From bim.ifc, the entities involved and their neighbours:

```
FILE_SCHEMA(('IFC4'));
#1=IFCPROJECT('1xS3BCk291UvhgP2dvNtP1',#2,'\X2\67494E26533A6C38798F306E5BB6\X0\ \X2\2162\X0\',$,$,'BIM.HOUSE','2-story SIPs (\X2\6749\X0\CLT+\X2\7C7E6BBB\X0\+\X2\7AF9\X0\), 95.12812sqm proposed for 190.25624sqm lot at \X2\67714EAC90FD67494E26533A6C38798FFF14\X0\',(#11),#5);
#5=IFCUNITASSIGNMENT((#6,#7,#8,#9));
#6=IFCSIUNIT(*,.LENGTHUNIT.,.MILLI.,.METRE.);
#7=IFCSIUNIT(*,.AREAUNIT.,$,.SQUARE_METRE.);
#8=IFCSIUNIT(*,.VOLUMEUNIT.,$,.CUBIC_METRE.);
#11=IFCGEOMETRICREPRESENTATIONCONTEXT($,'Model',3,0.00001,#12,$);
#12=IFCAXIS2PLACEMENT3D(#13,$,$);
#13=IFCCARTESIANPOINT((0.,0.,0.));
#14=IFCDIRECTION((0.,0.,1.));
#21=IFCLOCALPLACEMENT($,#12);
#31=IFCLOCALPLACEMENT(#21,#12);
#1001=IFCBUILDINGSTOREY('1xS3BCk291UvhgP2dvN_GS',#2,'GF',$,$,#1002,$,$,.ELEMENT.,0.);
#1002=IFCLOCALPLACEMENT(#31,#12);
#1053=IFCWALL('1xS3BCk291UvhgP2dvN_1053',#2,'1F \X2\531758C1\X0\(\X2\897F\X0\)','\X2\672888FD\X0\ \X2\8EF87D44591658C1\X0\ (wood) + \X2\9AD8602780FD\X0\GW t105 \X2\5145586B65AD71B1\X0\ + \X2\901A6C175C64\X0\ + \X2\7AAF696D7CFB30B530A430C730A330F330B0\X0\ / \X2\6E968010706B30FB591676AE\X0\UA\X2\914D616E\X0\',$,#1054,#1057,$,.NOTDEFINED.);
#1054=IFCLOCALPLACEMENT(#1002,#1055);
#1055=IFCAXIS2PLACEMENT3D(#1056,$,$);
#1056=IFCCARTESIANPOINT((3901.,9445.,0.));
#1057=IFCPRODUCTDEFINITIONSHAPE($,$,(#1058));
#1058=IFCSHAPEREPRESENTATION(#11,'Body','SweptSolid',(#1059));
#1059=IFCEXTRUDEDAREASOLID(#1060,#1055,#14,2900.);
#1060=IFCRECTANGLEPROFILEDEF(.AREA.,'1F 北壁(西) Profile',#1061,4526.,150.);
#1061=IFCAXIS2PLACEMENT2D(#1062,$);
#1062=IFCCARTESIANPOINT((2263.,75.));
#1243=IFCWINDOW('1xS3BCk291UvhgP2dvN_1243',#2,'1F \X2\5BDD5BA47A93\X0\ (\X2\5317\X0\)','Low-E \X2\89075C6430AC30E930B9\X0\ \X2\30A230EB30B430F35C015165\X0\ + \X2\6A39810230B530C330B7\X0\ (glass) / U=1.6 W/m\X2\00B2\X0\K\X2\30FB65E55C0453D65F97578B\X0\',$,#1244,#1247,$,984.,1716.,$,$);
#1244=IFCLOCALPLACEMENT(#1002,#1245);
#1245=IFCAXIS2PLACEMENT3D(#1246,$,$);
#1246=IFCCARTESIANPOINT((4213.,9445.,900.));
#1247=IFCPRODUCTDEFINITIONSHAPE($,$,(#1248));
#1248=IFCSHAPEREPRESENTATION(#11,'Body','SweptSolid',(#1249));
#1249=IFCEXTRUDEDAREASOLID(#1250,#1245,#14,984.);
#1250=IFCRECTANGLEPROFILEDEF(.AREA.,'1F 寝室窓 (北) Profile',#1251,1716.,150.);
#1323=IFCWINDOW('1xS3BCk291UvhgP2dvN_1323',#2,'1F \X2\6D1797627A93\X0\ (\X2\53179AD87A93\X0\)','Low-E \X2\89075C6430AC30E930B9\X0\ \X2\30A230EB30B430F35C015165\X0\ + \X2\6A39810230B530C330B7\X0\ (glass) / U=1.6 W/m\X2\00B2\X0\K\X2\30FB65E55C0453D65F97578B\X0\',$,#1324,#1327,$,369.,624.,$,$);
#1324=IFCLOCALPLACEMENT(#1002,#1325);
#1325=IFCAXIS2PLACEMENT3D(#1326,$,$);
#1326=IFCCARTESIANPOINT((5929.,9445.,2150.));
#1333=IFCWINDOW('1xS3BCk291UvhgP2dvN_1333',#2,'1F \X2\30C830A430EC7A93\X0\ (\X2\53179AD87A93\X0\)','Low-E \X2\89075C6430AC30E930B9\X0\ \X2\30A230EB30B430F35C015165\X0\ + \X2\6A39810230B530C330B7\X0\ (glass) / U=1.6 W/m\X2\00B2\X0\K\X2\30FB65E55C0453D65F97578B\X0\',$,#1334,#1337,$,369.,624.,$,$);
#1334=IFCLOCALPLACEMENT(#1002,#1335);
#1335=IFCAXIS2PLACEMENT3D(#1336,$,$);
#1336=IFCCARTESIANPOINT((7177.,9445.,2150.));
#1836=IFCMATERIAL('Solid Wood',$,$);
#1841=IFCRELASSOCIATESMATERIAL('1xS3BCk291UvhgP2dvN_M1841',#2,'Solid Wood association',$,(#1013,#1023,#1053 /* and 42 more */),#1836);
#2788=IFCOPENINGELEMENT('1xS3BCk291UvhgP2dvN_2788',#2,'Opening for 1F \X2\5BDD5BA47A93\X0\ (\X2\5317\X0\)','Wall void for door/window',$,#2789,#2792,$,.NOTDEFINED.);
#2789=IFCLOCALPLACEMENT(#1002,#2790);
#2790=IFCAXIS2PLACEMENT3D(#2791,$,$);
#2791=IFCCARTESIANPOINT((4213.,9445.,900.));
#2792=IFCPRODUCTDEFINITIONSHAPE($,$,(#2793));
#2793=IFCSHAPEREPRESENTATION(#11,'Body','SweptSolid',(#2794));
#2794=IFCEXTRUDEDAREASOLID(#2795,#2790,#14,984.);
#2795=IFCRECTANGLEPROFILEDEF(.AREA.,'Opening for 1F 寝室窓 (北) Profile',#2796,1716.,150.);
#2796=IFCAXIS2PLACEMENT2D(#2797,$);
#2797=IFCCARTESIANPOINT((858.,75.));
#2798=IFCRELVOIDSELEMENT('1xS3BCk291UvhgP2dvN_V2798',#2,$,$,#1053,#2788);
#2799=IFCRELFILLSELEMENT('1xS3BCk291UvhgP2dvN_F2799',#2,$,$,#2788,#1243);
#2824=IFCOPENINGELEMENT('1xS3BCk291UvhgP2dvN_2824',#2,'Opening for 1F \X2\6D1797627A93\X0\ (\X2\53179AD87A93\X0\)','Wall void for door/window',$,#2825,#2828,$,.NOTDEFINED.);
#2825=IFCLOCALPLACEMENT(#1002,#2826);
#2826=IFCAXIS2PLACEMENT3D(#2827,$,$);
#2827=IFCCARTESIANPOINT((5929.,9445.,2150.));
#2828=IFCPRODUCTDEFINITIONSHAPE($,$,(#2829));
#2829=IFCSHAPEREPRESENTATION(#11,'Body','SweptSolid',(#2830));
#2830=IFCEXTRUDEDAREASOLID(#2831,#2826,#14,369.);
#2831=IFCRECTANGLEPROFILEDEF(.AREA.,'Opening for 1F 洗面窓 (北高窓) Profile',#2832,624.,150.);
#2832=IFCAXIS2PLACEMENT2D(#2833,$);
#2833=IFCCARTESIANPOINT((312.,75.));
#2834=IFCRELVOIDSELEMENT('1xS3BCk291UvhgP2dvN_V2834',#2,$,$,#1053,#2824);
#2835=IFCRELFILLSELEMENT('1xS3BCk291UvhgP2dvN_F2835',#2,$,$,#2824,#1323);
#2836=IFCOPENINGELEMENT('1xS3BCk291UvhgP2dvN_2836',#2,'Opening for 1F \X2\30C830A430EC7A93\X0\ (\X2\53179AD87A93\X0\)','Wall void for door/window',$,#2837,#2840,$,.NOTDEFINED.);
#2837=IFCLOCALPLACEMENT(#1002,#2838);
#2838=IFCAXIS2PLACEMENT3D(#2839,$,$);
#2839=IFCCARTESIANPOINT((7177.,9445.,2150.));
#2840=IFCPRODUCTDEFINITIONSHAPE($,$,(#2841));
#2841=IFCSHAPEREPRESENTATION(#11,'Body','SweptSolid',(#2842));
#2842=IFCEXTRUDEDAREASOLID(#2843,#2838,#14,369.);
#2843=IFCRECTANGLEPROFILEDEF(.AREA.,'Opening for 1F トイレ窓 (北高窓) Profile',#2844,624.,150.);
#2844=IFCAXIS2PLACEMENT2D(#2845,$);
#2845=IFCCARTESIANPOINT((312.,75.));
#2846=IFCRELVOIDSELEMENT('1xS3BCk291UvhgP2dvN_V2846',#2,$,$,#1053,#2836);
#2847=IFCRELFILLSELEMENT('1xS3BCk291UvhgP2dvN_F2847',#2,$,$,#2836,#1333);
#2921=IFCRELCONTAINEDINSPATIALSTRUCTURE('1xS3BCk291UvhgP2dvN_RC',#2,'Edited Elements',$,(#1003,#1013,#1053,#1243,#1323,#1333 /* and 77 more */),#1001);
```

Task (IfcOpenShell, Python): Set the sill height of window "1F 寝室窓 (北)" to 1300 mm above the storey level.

```python
import numpy as np
import ifcopenshell
import ifcopenshell.api.geometry
import ifcopenshell.geom
import ifcopenshell.util.element
import ifcopenshell.util.placement
import ifcopenshell.util.shape
import ifcopenshell.util.unit

model = ifcopenshell.open("bim.ifc")
unit_scale = ifcopenshell.util.unit.calculate_unit_scale(model)

window = model.by_id(1243)
opening = window.FillsVoids[0].RelatingOpeningElement
storey = ifcopenshell.util.element.get_container(window, ifc_class="IfcBuildingStorey")
level = ifcopenshell.util.placement.get_local_placement(storey.ObjectPlacement)[2, 3]

# The opening's origin need not be at the sill, so measure its lowest point.
shape = ifcopenshell.geom.create_shape(ifcopenshell.geom.settings(), opening)
bottom = ifcopenshell.util.shape.get_shape_bottom_elevation(shape, shape.geometry) / unit_scale
dz = level + 1.3 / unit_scale - bottom

shift = np.array([0.0, 0.0, dz])
# The window is not placed relative to its opening, so move both.
for product in (opening, window):
    matrix = ifcopenshell.util.placement.get_local_placement(product.ObjectPlacement)
    matrix[:3, 3] += shift
    ifcopenshell.api.geometry.edit_object_placement(model, product=product, matrix=matrix, is_si=False)

print(f"moved by {dz * unit_scale:+.3f} m")

model.write("bim_updated.ifc")
```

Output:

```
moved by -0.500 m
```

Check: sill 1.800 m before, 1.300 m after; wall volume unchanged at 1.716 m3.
